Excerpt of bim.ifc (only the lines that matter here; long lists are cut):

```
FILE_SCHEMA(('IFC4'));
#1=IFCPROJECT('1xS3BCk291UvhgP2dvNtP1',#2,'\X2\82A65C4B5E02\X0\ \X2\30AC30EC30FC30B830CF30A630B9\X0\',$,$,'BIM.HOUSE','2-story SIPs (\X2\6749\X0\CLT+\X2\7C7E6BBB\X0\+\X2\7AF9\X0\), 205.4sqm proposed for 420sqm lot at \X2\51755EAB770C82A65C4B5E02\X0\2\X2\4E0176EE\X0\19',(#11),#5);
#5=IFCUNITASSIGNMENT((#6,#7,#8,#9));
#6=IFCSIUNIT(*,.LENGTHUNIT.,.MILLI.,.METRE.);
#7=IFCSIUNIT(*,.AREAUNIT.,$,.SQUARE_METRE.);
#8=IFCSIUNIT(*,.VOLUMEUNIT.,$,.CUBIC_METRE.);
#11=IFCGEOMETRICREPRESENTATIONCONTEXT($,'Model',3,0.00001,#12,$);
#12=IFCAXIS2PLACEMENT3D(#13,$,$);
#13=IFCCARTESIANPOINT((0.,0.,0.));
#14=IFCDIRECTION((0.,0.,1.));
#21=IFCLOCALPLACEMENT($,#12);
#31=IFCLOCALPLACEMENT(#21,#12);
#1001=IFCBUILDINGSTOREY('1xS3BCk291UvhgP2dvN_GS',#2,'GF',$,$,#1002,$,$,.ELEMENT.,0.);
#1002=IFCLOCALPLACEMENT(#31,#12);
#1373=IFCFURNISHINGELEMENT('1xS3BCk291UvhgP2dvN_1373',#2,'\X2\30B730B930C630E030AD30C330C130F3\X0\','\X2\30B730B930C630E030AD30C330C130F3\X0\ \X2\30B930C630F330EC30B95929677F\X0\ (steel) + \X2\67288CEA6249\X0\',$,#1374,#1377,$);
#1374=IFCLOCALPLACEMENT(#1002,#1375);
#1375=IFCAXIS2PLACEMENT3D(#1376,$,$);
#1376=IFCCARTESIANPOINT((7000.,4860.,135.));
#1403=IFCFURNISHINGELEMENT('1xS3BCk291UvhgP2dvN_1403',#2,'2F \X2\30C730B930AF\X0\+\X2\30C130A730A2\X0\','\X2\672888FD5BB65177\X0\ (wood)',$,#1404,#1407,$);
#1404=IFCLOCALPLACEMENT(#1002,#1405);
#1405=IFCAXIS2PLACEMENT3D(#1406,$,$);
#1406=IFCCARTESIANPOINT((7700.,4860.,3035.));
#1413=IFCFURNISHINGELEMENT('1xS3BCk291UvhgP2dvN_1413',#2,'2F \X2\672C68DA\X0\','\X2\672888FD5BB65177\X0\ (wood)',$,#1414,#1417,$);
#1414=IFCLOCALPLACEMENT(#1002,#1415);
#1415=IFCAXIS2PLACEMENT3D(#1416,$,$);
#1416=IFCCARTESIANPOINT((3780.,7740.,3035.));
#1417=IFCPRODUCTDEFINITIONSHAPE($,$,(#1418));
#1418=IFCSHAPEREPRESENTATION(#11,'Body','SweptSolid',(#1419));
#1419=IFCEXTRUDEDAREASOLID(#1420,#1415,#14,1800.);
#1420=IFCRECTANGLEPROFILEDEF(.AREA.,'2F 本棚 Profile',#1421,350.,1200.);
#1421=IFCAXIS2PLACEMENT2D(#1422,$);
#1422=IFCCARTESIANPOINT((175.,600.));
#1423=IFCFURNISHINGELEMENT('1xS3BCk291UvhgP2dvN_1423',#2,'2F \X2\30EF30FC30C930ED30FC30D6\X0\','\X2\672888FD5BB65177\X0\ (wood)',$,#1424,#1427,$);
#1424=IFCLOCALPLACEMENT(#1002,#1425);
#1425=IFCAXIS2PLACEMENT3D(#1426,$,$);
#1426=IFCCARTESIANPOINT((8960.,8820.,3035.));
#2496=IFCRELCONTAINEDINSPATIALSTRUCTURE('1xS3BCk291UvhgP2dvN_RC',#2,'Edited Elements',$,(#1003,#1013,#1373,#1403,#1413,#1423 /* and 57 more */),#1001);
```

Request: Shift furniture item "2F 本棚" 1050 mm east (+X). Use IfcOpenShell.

```python
import ifcopenshell
import ifcopenshell.api.geometry
import ifcopenshell.util.placement

model = ifcopenshell.open("bim.ifc")

item = model.by_guid("1xS3BCk291UvhgP2dvN_1413")
matrix = ifcopenshell.util.placement.get_local_placement(item.ObjectPlacement)
matrix[0, 3] += 1050.0
ifcopenshell.api.geometry.edit_object_placement(model, product=item, matrix=matrix, is_si=False)

print(ifcopenshell.util.placement.get_local_placement(item.ObjectPlacement).round(3) + 0.0)

model.write("bim_v2.ifc")
```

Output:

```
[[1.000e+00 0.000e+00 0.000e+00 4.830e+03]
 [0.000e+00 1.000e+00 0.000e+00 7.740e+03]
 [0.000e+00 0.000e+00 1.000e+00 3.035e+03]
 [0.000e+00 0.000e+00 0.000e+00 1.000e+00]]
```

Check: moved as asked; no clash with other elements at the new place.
